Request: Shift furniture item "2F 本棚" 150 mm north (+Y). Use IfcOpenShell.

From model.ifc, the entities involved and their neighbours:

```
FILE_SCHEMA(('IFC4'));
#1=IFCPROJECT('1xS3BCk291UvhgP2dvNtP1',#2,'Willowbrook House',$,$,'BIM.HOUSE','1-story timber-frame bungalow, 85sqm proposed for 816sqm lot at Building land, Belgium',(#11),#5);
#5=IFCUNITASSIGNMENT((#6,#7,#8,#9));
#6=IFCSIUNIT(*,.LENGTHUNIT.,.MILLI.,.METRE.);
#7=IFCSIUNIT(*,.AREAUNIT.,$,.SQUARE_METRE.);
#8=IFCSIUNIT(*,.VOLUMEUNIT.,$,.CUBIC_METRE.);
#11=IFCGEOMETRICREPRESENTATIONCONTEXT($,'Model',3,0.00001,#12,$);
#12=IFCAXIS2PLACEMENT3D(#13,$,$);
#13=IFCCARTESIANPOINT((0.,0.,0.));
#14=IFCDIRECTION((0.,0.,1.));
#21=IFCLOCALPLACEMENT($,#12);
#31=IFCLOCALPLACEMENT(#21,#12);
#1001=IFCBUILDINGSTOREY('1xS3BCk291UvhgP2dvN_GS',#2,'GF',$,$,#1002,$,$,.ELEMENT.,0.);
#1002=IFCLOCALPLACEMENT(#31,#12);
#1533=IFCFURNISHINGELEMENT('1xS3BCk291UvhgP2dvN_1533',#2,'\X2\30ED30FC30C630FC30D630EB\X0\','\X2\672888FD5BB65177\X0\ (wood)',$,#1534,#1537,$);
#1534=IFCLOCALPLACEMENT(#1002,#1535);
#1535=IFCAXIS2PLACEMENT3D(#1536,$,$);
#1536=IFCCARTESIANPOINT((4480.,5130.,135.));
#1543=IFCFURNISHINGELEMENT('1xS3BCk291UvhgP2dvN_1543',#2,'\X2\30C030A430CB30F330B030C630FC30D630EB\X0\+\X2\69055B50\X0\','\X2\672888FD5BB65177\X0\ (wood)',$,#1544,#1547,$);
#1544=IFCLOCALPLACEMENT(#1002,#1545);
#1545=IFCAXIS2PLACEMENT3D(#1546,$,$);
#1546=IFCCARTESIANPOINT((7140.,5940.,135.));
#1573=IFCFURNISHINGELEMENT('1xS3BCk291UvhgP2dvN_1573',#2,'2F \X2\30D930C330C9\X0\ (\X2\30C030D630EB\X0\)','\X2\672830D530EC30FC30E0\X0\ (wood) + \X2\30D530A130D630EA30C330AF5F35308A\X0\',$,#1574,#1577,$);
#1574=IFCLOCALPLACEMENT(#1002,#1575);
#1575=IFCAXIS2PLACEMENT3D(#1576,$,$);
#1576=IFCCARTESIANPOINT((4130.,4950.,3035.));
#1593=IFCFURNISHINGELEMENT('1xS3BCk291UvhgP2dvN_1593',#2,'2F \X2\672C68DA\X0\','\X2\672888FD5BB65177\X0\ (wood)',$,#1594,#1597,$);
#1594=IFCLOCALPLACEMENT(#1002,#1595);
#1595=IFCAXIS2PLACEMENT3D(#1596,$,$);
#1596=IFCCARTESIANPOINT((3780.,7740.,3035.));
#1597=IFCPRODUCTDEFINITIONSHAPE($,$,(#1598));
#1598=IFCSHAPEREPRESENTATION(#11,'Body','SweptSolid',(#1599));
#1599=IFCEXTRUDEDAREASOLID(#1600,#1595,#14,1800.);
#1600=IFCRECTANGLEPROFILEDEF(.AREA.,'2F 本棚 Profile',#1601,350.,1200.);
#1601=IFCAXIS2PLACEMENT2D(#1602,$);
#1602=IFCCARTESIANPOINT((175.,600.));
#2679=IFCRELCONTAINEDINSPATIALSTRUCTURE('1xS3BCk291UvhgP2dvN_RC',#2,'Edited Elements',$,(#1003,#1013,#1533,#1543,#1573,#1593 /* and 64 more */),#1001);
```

```python
import ifcopenshell
import ifcopenshell.api.geometry
import ifcopenshell.util.placement
import ifcopenshell.util.unit

model = ifcopenshell.open("model.ifc")
unit_scale = ifcopenshell.util.unit.calculate_unit_scale(model)

item = model.by_guid("1xS3BCk291UvhgP2dvN_1593")
matrix = ifcopenshell.util.placement.get_local_placement(item.ObjectPlacement)
matrix[1, 3] += 0.15 / unit_scale
ifcopenshell.api.geometry.edit_object_placement(model, product=item, matrix=matrix, is_si=False)

print(ifcopenshell.util.placement.get_local_placement(item.ObjectPlacement).round(3) + 0.0)

model.write("model_rev.ifc")
```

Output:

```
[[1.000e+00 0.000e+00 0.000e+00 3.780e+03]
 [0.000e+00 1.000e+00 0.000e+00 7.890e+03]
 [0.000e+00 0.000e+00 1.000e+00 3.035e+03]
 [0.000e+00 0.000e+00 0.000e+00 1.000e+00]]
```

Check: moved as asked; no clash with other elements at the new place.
